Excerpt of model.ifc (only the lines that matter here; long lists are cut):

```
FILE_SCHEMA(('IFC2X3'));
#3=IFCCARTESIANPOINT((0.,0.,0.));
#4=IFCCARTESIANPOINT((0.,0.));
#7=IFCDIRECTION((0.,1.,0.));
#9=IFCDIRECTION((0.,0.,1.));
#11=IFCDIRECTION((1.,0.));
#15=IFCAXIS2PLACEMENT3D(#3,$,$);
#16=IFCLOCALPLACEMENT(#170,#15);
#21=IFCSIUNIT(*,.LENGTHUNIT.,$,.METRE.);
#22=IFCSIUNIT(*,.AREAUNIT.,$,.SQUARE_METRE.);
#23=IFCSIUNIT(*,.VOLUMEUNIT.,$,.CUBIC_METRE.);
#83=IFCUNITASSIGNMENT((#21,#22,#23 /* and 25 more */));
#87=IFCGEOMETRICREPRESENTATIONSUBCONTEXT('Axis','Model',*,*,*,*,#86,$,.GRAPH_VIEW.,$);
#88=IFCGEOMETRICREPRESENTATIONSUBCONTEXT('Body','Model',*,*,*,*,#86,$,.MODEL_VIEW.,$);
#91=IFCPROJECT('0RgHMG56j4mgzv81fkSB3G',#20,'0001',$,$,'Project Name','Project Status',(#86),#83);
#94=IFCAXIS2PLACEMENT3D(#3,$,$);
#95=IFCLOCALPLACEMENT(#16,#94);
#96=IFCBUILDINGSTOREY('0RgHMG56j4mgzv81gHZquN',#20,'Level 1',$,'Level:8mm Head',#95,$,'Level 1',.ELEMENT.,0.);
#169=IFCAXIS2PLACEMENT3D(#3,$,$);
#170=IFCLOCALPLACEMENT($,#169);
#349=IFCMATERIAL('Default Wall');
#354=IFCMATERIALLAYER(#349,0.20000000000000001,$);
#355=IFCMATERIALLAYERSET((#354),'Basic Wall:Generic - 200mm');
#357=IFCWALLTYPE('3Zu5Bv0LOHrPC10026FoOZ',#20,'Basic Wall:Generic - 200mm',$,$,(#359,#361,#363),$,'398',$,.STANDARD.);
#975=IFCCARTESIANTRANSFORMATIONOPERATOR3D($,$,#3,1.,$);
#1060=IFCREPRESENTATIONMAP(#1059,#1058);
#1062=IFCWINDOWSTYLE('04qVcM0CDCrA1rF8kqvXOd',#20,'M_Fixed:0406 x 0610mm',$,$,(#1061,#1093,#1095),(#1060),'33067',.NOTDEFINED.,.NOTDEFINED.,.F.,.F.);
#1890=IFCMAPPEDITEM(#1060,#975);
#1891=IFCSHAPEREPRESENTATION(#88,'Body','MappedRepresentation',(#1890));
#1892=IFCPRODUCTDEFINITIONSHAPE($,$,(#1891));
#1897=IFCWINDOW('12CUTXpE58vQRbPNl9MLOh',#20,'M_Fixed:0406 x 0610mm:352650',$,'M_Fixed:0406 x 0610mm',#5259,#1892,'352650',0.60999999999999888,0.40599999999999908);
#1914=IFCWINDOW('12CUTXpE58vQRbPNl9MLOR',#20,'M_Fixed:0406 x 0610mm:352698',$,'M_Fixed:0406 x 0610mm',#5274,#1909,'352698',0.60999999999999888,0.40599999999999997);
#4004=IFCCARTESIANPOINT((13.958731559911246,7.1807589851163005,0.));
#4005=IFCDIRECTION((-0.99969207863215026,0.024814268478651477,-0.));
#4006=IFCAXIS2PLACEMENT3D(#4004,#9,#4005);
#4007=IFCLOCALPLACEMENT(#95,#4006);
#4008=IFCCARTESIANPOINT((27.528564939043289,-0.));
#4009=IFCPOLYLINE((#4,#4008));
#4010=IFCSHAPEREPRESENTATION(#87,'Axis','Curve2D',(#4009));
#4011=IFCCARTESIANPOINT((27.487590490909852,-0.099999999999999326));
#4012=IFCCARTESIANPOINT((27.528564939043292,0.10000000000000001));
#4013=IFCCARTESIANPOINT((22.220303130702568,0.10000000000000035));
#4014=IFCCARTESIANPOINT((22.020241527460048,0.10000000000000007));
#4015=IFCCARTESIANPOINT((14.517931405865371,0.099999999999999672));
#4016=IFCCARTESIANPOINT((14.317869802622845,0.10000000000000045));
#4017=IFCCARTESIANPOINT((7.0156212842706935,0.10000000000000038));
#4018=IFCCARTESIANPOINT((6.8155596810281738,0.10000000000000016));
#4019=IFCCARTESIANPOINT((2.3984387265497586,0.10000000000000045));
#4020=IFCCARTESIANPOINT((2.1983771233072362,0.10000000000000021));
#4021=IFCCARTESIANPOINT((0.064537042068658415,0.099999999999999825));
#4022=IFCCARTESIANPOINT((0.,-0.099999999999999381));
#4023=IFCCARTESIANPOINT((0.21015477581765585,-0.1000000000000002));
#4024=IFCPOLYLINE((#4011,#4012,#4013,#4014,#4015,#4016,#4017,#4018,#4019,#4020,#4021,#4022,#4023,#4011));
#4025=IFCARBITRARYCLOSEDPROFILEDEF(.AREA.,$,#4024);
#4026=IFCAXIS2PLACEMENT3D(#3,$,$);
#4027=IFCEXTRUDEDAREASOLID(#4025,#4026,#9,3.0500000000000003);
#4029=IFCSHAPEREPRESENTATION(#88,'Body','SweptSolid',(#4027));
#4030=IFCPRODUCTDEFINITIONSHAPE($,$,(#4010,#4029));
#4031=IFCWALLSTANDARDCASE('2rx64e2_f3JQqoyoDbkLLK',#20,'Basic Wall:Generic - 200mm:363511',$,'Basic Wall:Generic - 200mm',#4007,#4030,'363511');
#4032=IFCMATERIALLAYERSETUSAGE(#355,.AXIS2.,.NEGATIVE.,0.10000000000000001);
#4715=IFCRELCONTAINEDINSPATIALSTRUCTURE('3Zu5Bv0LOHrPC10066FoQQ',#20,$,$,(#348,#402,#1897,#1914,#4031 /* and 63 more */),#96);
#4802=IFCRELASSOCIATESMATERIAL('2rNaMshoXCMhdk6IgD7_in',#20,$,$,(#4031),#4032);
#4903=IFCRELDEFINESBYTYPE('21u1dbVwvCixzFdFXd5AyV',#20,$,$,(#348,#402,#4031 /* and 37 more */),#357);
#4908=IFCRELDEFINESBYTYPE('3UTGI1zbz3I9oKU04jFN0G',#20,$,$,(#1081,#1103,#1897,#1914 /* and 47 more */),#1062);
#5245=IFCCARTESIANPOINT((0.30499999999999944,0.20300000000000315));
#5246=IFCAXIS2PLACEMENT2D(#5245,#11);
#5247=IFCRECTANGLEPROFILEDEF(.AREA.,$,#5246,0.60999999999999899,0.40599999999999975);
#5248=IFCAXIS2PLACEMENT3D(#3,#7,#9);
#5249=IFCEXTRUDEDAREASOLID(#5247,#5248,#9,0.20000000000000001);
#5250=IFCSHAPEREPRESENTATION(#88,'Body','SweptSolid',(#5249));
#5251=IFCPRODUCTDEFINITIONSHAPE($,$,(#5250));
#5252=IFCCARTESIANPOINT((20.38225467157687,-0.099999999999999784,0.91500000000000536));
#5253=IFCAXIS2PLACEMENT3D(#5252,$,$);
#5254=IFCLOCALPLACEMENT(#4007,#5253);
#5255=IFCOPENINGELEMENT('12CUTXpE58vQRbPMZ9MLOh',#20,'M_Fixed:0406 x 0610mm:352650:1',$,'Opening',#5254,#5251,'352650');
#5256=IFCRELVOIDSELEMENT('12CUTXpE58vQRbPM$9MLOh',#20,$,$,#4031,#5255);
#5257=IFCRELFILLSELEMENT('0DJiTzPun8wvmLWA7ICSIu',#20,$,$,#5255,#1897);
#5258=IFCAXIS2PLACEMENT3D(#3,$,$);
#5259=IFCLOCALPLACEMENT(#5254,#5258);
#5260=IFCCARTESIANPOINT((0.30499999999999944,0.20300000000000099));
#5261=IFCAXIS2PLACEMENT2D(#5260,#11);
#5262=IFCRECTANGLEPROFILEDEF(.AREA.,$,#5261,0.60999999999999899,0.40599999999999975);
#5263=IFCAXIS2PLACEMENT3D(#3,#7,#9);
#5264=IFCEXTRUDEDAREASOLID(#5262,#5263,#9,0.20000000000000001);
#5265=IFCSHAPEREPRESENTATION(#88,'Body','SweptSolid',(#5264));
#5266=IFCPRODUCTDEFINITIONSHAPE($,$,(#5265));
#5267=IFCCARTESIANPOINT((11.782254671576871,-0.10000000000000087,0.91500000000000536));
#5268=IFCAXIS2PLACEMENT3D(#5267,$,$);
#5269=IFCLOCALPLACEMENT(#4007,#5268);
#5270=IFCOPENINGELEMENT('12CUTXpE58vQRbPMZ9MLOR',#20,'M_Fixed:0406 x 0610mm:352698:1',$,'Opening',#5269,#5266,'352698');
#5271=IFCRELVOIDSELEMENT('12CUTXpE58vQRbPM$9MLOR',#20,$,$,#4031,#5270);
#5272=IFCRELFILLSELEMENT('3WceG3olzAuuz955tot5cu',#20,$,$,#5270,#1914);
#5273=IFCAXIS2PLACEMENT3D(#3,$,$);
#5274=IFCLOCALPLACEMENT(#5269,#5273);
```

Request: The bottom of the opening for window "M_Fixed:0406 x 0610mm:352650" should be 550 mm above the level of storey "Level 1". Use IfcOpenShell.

```python
import numpy as np
import ifcopenshell
import ifcopenshell.api.geometry
import ifcopenshell.geom
import ifcopenshell.util.element
import ifcopenshell.util.placement
import ifcopenshell.util.shape
import ifcopenshell.util.unit

model = ifcopenshell.open("model.ifc")
unit_scale = ifcopenshell.util.unit.calculate_unit_scale(model)

window = model.by_id(1897)
opening = window.FillsVoids[0].RelatingOpeningElement
storey = ifcopenshell.util.element.get_container(window, ifc_class="IfcBuildingStorey")
level = ifcopenshell.util.placement.get_local_placement(storey.ObjectPlacement)[2, 3]

# The opening's origin need not be at the sill, so measure its lowest point.
shape = ifcopenshell.geom.create_shape(ifcopenshell.geom.settings(), opening)
bottom = ifcopenshell.util.shape.get_shape_bottom_elevation(shape, shape.geometry) / unit_scale
dz = level + 0.55 / unit_scale - bottom

shift = np.array([0.0, 0.0, dz])
# The window is placed relative to its opening, so it follows when the opening moves.
matrix = ifcopenshell.util.placement.get_local_placement(opening.ObjectPlacement)
matrix[:3, 3] += shift
ifcopenshell.api.geometry.edit_object_placement(
    model, product=opening, matrix=matrix, is_si=False, should_transform_children=True
)

print(f"moved by {dz * unit_scale:+.3f} m")

model.write("model_edited.ifc")
```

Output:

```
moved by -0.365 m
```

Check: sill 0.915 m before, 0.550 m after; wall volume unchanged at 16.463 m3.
